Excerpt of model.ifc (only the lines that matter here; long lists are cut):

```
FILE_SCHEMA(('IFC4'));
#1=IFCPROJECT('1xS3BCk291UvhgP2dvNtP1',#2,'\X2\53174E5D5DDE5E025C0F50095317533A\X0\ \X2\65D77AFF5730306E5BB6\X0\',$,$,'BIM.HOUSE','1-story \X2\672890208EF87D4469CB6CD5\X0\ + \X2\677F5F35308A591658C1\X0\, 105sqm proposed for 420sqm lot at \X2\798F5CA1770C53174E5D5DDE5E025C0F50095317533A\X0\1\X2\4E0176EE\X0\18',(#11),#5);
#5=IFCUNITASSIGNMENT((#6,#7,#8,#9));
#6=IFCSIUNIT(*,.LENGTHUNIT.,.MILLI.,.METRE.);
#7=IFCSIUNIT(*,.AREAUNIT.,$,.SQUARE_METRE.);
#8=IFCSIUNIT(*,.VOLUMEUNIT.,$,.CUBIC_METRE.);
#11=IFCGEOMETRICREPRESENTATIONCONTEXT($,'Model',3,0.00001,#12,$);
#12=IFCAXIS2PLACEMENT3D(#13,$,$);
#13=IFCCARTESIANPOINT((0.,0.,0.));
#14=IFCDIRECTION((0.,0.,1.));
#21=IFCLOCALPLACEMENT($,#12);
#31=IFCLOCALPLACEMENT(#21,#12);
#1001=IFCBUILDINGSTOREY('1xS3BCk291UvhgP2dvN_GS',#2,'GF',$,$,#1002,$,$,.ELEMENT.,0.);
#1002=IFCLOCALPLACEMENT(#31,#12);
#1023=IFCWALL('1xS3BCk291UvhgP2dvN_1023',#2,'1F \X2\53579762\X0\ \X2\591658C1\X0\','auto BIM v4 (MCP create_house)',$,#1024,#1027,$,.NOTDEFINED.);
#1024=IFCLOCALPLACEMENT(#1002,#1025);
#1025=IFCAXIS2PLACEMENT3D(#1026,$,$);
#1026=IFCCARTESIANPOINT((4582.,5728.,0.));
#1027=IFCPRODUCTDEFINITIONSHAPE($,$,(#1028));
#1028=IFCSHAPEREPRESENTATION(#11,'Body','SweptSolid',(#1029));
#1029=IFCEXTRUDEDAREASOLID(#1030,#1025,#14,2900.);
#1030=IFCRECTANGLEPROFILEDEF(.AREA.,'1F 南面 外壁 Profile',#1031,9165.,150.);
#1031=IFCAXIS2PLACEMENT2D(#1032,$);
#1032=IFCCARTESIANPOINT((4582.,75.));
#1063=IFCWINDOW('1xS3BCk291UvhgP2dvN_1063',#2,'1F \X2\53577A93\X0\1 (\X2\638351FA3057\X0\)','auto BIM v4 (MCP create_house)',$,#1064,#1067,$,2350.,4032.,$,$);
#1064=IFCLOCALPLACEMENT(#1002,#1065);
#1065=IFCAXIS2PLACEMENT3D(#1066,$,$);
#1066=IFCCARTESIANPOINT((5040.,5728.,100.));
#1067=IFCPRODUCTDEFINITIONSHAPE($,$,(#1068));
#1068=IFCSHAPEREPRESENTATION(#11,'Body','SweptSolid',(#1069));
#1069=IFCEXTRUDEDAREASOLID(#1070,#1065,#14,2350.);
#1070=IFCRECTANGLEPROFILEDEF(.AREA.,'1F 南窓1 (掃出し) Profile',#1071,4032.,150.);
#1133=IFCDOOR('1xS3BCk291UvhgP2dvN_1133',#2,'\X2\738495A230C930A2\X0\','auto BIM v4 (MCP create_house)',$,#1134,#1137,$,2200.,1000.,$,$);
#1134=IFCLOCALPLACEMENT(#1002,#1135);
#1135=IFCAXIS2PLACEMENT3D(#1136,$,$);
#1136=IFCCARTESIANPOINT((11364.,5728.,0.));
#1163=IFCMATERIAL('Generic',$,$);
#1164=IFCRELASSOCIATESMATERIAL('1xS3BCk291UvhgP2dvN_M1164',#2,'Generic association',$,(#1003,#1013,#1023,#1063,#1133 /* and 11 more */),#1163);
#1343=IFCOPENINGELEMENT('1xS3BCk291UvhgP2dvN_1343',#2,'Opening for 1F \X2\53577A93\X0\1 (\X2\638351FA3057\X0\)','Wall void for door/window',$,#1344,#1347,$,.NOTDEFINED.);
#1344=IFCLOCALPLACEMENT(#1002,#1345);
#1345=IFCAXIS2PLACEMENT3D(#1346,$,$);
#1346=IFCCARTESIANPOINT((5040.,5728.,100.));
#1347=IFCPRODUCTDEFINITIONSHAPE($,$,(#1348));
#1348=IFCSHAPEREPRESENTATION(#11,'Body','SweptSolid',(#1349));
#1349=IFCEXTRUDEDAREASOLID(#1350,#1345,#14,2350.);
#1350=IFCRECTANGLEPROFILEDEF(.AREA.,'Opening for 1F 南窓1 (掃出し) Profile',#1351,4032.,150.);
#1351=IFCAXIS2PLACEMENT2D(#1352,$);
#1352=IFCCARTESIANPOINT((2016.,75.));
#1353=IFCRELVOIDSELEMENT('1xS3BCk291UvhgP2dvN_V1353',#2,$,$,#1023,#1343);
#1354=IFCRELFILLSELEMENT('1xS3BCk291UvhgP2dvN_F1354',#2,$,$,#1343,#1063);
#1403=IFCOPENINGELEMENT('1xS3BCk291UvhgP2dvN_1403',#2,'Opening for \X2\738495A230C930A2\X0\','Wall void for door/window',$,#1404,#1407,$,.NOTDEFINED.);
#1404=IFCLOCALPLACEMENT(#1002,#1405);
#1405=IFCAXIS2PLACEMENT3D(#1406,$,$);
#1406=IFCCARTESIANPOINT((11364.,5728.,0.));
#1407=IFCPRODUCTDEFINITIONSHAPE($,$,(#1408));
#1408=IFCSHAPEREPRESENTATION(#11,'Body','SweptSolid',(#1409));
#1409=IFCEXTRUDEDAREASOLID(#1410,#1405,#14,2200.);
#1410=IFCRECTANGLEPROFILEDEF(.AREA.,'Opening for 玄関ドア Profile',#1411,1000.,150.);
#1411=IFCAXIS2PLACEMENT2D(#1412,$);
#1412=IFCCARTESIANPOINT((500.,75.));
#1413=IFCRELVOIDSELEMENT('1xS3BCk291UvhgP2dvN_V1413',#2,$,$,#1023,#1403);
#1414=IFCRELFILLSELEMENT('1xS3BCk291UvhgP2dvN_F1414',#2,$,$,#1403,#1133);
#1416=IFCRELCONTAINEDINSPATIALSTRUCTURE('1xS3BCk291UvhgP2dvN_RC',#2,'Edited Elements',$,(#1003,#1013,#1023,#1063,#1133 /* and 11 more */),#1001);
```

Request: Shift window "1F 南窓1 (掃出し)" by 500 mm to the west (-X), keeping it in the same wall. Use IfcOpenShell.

```python
import ifcopenshell
import ifcopenshell.api.geometry
import ifcopenshell.util.placement
import ifcopenshell.util.unit

model = ifcopenshell.open("model.ifc")
unit_scale = ifcopenshell.util.unit.calculate_unit_scale(model)

window = model.by_guid("1xS3BCk291UvhgP2dvN_1063")
opening = window.FillsVoids[0].RelatingOpeningElement
wall = opening.VoidsElements[0].RelatingBuildingElement

wall_matrix = ifcopenshell.util.placement.get_local_placement(wall.ObjectPlacement)
shift = wall_matrix[:3, 0] * -0.5 / unit_scale
before = ifcopenshell.util.placement.get_local_placement(window.ObjectPlacement)[:3, 3].copy()

# The window is not placed relative to its opening, so move both.
for product in (opening, window):
    matrix = ifcopenshell.util.placement.get_local_placement(product.ObjectPlacement)
    matrix[:3, 3] += shift
    ifcopenshell.api.geometry.edit_object_placement(model, product=product, matrix=matrix, is_si=False)

after = ifcopenshell.util.placement.get_local_placement(window.ObjectPlacement)[:3, 3]
print("window moved by", (after - before).round(3) + 0.0)

model.write("model_rev.ifc")
```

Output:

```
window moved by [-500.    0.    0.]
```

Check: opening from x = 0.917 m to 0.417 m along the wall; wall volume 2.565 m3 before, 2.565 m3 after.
